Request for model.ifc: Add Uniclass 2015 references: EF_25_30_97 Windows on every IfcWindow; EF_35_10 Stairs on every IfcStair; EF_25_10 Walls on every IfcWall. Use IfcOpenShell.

First a look at what the model holds.

```python
import ifcopenshell

model = ifcopenshell.open("model.ifc")
print(model.schema)
print("classifications:", [c.Name for c in model.by_type("IfcClassification")])
for ifc_class in ("IfcDoor", "IfcRoof", "IfcStair", "IfcWall", "IfcWindow"):
    print(ifc_class, len(model.by_type(ifc_class)))
```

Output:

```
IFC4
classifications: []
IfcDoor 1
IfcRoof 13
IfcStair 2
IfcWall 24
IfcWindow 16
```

```python
import ifcopenshell
import ifcopenshell.api.classification

model = ifcopenshell.open("model.ifc")

system = ifcopenshell.api.classification.add_classification(model, classification="Uniclass 2015")

codes = {
    "IfcWindow": ("EF_25_30_97", "Windows"),
    "IfcStair": ("EF_35_10", "Stairs"),
    "IfcWall": ("EF_25_10", "Walls"),
}
for ifc_class, (code, name) in codes.items():
    products = model.by_type(ifc_class)
    ifcopenshell.api.classification.add_reference(
        model, products=products, classification=system, identification=code, name=name
    )
    print(code, len(products))

model.write("model_updated.ifc")
```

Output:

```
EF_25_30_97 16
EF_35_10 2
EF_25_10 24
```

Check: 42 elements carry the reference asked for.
